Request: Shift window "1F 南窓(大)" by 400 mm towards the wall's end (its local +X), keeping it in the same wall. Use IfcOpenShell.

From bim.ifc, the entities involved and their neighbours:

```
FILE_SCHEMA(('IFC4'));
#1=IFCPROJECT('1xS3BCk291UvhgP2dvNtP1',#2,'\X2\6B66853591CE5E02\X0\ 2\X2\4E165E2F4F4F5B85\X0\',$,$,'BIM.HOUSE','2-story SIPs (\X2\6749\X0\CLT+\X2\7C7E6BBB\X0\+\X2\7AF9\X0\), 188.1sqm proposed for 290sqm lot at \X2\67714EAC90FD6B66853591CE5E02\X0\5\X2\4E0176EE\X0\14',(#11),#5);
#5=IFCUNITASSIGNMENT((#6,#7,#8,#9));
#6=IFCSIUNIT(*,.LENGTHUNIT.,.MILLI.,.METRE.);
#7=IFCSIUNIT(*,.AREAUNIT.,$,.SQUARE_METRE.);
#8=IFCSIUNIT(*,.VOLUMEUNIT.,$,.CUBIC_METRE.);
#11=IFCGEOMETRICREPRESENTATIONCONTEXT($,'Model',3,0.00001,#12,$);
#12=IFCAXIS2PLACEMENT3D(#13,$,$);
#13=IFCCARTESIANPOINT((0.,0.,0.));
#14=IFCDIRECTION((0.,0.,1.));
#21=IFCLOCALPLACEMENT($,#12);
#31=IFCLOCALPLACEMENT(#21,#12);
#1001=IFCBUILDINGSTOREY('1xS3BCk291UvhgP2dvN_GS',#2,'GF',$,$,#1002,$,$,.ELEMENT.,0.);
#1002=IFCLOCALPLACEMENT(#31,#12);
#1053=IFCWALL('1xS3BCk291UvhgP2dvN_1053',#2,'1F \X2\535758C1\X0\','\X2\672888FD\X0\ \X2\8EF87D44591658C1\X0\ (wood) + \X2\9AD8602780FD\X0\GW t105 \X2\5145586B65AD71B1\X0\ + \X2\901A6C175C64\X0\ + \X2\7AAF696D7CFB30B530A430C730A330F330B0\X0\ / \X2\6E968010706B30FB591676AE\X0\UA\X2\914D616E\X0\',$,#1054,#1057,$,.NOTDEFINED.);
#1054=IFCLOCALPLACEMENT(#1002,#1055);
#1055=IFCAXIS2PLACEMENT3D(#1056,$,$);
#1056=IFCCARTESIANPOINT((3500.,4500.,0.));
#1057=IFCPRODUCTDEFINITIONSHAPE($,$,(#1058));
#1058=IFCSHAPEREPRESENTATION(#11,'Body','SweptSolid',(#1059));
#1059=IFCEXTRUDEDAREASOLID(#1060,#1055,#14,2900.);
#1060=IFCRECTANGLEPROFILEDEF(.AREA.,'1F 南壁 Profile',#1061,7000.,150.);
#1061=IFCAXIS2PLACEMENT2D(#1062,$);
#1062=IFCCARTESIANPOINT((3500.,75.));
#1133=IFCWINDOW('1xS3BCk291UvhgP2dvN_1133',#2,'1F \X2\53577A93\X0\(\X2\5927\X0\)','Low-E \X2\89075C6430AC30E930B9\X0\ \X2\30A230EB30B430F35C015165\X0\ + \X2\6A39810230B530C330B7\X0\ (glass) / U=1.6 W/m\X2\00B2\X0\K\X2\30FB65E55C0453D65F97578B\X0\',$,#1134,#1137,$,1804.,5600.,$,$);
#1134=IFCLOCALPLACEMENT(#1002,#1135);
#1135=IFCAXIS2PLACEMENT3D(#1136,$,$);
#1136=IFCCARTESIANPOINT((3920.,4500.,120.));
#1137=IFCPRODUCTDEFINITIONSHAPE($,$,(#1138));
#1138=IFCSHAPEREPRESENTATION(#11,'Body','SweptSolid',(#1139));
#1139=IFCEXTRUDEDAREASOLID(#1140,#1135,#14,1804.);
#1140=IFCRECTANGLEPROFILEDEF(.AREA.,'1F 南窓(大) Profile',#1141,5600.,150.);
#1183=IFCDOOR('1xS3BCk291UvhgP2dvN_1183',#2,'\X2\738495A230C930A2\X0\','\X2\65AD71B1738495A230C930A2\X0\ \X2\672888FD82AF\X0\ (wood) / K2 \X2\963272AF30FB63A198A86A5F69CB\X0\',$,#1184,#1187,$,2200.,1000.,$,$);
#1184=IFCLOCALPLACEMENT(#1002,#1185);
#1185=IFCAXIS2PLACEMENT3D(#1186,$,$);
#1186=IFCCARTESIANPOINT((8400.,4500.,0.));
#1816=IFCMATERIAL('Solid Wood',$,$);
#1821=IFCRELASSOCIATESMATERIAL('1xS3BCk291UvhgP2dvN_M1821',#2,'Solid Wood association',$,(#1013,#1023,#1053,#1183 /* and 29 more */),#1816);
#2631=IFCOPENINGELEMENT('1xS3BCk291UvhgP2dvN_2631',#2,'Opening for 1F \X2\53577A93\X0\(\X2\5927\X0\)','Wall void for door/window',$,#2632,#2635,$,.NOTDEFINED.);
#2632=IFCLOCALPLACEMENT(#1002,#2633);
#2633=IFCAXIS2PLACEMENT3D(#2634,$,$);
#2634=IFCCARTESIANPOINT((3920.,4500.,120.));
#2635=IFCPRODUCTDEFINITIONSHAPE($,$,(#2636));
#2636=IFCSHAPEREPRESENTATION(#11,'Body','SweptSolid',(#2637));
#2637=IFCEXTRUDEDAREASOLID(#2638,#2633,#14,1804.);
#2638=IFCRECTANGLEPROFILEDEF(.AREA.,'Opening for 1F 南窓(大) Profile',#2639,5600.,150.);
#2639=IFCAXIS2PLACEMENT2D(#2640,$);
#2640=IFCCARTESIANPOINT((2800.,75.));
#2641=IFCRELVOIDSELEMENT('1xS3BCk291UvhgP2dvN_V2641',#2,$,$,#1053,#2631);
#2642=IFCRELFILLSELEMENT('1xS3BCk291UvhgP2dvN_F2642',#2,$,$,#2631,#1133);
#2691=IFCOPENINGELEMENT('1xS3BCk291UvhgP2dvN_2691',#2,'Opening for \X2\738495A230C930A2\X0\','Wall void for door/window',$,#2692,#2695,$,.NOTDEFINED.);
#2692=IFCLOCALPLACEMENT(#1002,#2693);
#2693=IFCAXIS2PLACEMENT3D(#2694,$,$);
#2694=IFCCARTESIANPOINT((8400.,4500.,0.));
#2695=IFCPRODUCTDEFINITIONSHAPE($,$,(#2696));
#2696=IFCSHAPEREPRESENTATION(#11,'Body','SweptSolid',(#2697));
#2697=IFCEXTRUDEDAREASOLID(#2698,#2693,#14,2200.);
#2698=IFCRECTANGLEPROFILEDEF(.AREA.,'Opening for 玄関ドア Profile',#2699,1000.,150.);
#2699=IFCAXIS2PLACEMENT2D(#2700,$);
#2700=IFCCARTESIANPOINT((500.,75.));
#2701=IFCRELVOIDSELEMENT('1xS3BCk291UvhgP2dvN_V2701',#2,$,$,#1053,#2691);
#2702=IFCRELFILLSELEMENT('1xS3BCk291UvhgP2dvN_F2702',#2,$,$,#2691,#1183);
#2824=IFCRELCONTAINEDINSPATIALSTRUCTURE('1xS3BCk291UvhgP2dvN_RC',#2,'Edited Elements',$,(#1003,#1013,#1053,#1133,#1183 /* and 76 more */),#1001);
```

```python
import ifcopenshell
import ifcopenshell.api.geometry
import ifcopenshell.util.placement
import ifcopenshell.util.unit

model = ifcopenshell.open("bim.ifc")
unit_scale = ifcopenshell.util.unit.calculate_unit_scale(model)

window = model.by_guid("1xS3BCk291UvhgP2dvN_1133")
opening = window.FillsVoids[0].RelatingOpeningElement
wall = opening.VoidsElements[0].RelatingBuildingElement

wall_matrix = ifcopenshell.util.placement.get_local_placement(wall.ObjectPlacement)
shift = wall_matrix[:3, 0] * 0.4 / unit_scale
before = ifcopenshell.util.placement.get_local_placement(window.ObjectPlacement)[:3, 3].copy()

# The window is not placed relative to its opening, so move both.
for product in (opening, window):
    matrix = ifcopenshell.util.placement.get_local_placement(product.ObjectPlacement)
    matrix[:3, 3] += shift
    ifcopenshell.api.geometry.edit_object_placement(model, product=product, matrix=matrix, is_si=False)

after = ifcopenshell.util.placement.get_local_placement(window.ObjectPlacement)[:3, 3]
print("window moved by", (after - before).round(3) + 0.0)

model.write("bim-out.ifc")
```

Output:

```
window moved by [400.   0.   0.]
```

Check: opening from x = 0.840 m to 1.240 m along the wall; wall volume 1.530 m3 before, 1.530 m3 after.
